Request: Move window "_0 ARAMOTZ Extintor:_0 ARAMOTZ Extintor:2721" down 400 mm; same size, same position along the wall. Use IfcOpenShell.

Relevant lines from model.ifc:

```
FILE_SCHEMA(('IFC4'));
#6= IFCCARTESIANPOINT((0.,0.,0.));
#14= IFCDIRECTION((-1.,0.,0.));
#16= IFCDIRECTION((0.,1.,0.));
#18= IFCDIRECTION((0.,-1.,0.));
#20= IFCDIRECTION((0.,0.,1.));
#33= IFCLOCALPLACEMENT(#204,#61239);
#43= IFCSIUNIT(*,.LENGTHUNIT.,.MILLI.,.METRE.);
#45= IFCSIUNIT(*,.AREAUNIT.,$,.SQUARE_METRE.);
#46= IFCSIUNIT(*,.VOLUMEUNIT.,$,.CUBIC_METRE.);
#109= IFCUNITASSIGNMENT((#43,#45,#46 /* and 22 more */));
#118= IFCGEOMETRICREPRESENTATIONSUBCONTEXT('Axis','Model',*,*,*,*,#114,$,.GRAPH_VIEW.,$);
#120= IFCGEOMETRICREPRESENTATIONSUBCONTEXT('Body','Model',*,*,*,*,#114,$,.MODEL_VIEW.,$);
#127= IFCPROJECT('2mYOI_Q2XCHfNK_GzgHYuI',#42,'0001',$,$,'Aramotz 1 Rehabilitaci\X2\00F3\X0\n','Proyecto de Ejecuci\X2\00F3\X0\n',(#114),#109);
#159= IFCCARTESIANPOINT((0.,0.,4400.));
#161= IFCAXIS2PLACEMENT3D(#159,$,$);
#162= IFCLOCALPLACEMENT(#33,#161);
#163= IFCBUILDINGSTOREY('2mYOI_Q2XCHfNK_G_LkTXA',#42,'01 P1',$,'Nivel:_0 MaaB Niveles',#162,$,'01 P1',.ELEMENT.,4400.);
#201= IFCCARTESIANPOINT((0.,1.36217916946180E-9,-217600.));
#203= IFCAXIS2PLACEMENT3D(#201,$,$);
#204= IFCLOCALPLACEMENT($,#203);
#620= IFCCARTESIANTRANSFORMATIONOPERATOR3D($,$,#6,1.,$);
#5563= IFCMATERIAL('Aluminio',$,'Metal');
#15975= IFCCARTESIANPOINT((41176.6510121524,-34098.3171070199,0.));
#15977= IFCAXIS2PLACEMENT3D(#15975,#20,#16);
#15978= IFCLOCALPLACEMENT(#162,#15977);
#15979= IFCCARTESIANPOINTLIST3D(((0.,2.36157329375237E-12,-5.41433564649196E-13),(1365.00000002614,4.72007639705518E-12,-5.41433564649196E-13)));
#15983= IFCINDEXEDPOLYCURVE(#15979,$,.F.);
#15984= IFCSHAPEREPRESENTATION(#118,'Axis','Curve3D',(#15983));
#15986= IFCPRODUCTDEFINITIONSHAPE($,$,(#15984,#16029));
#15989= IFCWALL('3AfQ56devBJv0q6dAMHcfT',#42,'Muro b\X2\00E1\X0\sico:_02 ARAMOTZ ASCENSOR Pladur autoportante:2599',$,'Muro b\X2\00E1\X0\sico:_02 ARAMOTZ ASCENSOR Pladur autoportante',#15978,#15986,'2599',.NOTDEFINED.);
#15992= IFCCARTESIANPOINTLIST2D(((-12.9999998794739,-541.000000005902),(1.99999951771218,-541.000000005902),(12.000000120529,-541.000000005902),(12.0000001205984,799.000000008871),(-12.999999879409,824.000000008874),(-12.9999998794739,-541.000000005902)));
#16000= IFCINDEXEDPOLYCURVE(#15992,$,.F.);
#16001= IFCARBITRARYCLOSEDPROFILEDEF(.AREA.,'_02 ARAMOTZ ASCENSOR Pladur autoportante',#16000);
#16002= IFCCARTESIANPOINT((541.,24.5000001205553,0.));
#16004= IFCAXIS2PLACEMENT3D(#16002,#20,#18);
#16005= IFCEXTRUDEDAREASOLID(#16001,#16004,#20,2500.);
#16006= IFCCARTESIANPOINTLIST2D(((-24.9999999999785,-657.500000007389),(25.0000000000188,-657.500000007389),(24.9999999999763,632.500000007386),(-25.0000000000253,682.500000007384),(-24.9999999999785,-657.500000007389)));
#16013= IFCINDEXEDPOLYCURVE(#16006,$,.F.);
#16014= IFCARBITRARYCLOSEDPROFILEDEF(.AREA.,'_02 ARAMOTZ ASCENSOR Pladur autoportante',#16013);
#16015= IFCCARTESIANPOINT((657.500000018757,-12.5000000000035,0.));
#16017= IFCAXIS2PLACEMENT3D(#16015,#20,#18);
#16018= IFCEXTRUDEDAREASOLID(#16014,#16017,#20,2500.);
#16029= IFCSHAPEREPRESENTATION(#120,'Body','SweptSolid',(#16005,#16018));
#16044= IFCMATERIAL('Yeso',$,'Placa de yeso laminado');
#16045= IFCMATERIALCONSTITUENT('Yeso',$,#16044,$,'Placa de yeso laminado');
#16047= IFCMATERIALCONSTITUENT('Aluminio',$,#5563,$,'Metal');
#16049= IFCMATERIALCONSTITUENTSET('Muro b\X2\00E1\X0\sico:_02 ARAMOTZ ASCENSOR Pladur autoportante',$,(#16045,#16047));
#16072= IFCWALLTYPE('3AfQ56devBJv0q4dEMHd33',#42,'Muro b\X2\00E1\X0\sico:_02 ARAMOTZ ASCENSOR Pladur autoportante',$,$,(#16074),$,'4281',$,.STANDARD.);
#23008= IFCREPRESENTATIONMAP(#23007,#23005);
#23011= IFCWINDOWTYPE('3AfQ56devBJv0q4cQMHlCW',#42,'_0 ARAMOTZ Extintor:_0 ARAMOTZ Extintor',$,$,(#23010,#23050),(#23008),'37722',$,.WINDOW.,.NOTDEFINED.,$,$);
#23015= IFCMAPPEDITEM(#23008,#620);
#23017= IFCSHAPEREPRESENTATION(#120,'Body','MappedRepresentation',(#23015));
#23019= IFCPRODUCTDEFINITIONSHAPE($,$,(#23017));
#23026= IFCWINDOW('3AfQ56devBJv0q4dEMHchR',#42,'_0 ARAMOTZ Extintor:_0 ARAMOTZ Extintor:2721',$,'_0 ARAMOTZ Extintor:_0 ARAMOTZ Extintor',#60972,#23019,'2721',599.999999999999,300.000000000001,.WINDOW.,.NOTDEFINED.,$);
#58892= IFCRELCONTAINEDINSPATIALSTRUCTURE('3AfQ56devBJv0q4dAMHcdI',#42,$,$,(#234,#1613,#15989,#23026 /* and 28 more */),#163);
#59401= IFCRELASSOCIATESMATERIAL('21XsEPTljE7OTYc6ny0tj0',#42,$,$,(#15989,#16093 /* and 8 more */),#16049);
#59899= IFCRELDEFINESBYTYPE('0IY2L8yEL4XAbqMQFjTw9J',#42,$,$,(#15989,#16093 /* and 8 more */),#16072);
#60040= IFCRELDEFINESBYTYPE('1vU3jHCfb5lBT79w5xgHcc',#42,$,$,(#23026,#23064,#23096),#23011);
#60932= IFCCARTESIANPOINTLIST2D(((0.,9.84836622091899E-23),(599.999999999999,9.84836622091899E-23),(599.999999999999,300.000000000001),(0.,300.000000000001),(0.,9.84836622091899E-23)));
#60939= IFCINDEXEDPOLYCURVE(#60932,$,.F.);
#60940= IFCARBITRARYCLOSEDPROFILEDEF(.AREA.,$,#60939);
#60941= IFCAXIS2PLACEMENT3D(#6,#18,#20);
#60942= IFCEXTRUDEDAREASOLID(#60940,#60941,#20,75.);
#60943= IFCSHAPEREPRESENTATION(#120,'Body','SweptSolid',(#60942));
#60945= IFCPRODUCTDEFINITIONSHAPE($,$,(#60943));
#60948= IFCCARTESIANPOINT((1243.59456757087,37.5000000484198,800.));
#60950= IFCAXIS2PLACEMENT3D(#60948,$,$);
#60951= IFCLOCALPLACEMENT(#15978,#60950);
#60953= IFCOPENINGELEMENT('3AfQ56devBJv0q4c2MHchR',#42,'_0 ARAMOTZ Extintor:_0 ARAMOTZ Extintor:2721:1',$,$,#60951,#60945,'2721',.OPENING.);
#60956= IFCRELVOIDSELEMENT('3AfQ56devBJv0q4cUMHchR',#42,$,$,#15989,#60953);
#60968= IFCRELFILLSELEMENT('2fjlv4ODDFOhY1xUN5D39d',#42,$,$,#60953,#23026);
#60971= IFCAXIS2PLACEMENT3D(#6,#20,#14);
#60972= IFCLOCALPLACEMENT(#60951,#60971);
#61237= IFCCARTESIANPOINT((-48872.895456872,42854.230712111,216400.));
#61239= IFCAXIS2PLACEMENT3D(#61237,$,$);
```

```python
import numpy as np
import ifcopenshell
import ifcopenshell.api.geometry
import ifcopenshell.util.placement
import ifcopenshell.util.unit

model = ifcopenshell.open("model.ifc")
unit_scale = ifcopenshell.util.unit.calculate_unit_scale(model)

window = model.by_guid("3AfQ56devBJv0q4dEMHchR")
opening = window.FillsVoids[0].RelatingOpeningElement
dz = -0.4 / unit_scale

shift = np.array([0.0, 0.0, dz])
# The window is placed relative to its opening, so it follows when the opening moves.
matrix = ifcopenshell.util.placement.get_local_placement(opening.ObjectPlacement)
matrix[:3, 3] += shift
ifcopenshell.api.geometry.edit_object_placement(
    model, product=opening, matrix=matrix, is_si=False, should_transform_children=True
)

print(f"moved by {dz * unit_scale:+.3f} m")

model.write("model-out.ifc")
```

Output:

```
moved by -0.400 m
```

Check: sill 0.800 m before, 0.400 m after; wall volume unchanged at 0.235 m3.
